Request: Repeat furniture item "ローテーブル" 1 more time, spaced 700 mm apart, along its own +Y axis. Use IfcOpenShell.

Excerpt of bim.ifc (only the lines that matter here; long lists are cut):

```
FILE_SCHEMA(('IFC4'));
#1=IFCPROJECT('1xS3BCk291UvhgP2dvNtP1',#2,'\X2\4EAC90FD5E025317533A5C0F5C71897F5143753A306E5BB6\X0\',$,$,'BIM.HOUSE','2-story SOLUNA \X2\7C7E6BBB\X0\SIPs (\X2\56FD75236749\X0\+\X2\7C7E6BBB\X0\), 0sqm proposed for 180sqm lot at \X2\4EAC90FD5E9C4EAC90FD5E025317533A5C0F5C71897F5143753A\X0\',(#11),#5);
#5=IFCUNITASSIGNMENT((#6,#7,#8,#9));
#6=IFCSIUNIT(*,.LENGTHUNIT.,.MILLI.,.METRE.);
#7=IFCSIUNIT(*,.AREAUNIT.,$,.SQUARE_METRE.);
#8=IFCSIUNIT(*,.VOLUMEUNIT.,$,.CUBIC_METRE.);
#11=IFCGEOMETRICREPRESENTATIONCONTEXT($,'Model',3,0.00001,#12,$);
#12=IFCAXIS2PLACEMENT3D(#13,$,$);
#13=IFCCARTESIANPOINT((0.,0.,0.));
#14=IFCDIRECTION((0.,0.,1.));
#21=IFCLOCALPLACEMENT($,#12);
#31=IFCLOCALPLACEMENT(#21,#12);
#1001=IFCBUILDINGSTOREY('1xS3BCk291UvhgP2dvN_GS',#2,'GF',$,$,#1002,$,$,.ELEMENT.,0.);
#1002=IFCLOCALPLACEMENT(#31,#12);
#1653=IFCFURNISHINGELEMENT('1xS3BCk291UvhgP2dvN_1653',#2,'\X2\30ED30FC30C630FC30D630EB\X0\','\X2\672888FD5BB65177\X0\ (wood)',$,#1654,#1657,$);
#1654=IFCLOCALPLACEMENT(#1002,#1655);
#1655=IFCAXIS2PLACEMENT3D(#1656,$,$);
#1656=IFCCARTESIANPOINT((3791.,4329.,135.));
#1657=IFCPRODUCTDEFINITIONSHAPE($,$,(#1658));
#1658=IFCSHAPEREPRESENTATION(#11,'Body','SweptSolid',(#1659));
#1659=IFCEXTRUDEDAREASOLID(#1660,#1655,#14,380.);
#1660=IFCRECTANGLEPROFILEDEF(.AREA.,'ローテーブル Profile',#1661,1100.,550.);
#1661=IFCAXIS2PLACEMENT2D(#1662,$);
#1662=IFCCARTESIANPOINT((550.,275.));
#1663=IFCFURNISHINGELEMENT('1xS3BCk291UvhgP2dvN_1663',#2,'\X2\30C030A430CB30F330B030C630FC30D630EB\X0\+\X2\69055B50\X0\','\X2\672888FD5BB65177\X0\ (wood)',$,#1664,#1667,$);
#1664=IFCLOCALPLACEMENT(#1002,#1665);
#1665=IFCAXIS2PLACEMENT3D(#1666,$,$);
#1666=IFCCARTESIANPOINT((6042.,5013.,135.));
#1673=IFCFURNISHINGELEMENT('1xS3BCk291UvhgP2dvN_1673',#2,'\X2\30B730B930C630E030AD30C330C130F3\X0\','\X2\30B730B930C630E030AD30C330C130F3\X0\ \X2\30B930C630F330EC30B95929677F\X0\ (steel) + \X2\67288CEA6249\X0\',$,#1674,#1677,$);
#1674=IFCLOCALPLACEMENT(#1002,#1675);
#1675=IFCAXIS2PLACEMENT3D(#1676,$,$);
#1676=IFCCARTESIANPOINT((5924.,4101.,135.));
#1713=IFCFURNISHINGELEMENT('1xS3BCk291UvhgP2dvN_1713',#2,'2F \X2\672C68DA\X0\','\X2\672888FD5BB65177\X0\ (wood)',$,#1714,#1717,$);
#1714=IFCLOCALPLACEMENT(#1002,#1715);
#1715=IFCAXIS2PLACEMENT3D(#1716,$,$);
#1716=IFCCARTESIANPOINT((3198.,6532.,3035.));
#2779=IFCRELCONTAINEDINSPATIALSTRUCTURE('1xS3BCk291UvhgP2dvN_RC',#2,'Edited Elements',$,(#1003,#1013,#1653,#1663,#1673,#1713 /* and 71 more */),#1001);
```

```python
import ifcopenshell
import ifcopenshell.api.geometry
import ifcopenshell.api.root
import ifcopenshell.util.element
import ifcopenshell.util.placement

model = ifcopenshell.open("bim.ifc")


def reuse_history(source, copy):
    """copy_class also copies each property set's owner history, people and application; keep the originals."""
    for rel in copy.IsDefinedBy:
        if rel.is_a("IfcRelDefinesByProperties") and (history := rel.RelatingPropertyDefinition.OwnerHistory):
            rel.RelatingPropertyDefinition.OwnerHistory = source.OwnerHistory
            ifcopenshell.util.element.remove_deep2(model, history)


source = model.by_guid("1xS3BCk291UvhgP2dvN_1653")
base = ifcopenshell.util.placement.get_local_placement(source.ObjectPlacement)
step = base[:3, 1] * 700.0

for i in range(1, 2):
    copy = ifcopenshell.api.root.copy_class(model, product=source)
    copy.Representation = ifcopenshell.util.element.copy_deep(
        model, source.Representation, exclude=["IfcGeometricRepresentationContext", "IfcRepresentationMap"]
    )
    reuse_history(source, copy)
    matrix = base.copy()
    matrix[:3, 3] += i * step
    print("added at", matrix[:3, 3].round(3) + 0.0)
    ifcopenshell.api.geometry.edit_object_placement(model, product=copy, matrix=matrix, is_si=False)

model.write("bim_updated.ifc")
```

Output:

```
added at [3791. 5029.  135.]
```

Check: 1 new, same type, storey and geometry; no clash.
